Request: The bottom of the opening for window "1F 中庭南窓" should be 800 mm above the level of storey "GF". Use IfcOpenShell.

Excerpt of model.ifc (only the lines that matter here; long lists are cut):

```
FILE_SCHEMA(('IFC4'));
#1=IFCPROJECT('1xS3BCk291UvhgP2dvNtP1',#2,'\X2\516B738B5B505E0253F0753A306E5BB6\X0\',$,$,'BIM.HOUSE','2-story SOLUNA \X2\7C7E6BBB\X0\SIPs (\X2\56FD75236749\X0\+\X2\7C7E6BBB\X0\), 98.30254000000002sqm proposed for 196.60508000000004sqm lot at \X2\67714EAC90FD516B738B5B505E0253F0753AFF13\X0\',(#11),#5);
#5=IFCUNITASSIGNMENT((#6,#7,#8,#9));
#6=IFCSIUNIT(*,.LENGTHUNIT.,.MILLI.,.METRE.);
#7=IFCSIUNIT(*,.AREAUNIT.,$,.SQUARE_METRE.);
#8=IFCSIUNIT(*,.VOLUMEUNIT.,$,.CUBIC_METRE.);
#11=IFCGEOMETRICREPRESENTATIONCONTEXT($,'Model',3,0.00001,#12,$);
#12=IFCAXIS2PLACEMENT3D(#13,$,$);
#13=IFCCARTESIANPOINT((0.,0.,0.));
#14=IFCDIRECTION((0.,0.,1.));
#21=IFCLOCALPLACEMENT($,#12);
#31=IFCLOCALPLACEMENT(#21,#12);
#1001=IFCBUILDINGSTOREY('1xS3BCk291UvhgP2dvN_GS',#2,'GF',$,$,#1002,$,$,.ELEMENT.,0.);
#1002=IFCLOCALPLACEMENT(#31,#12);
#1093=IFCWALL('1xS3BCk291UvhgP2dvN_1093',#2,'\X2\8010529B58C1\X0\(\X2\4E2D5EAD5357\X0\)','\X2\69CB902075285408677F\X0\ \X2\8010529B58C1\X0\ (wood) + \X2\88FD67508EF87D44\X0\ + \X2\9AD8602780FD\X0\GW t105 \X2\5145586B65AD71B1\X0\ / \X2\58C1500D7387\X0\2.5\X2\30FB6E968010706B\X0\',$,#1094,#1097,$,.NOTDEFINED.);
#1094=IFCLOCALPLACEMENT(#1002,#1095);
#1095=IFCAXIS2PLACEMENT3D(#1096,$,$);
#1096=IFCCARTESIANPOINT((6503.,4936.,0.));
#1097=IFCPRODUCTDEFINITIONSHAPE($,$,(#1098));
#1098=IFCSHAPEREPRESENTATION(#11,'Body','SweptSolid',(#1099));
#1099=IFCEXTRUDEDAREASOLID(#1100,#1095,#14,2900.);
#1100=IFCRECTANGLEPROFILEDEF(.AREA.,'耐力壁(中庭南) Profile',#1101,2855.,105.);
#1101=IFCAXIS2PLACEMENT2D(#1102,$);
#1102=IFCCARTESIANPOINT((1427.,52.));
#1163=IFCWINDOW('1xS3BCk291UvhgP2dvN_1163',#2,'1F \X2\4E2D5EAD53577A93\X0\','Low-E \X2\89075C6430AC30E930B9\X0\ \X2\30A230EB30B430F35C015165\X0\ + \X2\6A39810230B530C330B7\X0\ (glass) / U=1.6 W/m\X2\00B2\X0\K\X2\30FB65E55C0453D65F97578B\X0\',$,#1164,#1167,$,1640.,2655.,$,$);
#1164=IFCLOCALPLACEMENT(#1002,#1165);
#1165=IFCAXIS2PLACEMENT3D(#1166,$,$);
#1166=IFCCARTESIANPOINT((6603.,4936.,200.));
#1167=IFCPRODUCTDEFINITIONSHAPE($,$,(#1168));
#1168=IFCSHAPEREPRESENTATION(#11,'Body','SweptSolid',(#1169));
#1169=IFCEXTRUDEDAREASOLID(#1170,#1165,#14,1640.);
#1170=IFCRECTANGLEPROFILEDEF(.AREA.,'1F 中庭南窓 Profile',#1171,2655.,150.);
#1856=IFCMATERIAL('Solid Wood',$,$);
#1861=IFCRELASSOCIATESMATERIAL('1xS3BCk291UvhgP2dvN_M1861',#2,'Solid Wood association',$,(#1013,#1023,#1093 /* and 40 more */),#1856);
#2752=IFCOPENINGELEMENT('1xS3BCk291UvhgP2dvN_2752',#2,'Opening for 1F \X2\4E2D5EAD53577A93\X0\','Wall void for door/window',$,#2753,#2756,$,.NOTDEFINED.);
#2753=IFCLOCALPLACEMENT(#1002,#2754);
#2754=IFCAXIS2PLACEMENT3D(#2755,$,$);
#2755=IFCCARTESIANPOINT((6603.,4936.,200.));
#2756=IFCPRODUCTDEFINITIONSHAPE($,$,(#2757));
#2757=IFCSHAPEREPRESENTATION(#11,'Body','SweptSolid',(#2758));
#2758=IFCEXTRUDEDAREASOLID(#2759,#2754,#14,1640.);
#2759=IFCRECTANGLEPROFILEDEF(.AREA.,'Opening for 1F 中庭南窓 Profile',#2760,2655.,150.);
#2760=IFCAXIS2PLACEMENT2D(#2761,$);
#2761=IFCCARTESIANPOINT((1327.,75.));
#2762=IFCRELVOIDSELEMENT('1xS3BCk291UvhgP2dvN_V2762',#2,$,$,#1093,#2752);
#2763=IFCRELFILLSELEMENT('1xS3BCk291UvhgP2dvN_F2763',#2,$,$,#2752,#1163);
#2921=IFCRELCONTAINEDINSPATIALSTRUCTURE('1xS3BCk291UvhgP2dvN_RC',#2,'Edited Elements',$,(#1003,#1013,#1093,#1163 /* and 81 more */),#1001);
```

```python
import numpy as np
import ifcopenshell
import ifcopenshell.api.geometry
import ifcopenshell.geom
import ifcopenshell.util.element
import ifcopenshell.util.placement
import ifcopenshell.util.shape
import ifcopenshell.util.unit

model = ifcopenshell.open("model.ifc")
unit_scale = ifcopenshell.util.unit.calculate_unit_scale(model)

window = model.by_id(1163)
opening = window.FillsVoids[0].RelatingOpeningElement
storey = ifcopenshell.util.element.get_container(window, ifc_class="IfcBuildingStorey")
level = ifcopenshell.util.placement.get_local_placement(storey.ObjectPlacement)[2, 3]

# The opening's origin need not be at the sill, so measure its lowest point.
shape = ifcopenshell.geom.create_shape(ifcopenshell.geom.settings(), opening)
bottom = ifcopenshell.util.shape.get_shape_bottom_elevation(shape, shape.geometry) / unit_scale
dz = level + 800.0 - bottom

shift = np.array([0.0, 0.0, dz])
# The window is not placed relative to its opening, so move both.
for product in (opening, window):
    matrix = ifcopenshell.util.placement.get_local_placement(product.ObjectPlacement)
    matrix[:3, 3] += shift
    ifcopenshell.api.geometry.edit_object_placement(model, product=product, matrix=matrix, is_si=False)

print(f"moved by {dz * unit_scale:+.3f} m")

model.write("model_updated.ifc")
```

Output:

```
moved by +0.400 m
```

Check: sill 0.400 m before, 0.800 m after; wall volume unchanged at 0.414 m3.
